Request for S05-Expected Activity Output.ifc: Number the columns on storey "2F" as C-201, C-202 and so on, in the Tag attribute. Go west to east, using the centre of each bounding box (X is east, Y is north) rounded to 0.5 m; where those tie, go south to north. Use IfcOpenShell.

First a look at what the model holds.

```python
import ifcopenshell
import ifcopenshell.util.element
import ifcopenshell.util.placement

model = ifcopenshell.open("S05-Expected Activity Output.ifc")
print(model.schema)
storey = next(s for s in model.by_type("IfcBuildingStorey") if s.Name == "2F")
columns = [e for e in ifcopenshell.util.element.get_decomposition(storey) if e.is_a("IfcColumn")]
for e in sorted(columns, key=lambda e: e.id()):
    origin = ifcopenshell.util.placement.get_local_placement(e.ObjectPlacement)[:3, 3]
    print(e.id(), e.Tag, e.Name, origin.round(2) + 0.0, sep=" | ")
```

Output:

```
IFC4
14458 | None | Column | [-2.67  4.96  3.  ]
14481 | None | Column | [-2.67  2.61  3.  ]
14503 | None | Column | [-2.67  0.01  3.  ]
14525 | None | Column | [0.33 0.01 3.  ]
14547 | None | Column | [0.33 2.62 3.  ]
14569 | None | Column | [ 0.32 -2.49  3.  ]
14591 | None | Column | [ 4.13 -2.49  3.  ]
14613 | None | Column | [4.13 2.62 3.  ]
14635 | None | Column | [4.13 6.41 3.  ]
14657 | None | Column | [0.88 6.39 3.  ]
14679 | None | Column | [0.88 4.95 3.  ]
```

```python
import ifcopenshell
import ifcopenshell.geom
import ifcopenshell.util.element
import ifcopenshell.util.shape

model = ifcopenshell.open("S05-Expected Activity Output.ifc")
settings = ifcopenshell.geom.settings()
settings.set("use-world-coords", True)


def centre(element):
    shape = ifcopenshell.geom.create_shape(settings, element)
    return ifcopenshell.util.shape.get_bbox_centroid(shape.geometry)


storey = next(s for s in model.by_type("IfcBuildingStorey") if s.Name == "2F")
columns = [e for e in ifcopenshell.util.element.get_decomposition(storey) if e.is_a("IfcColumn")]

# Insertion points can sit at a corner or the storey origin, so sort by the geometry (in metres).
centres = {e: centre(e) for e in columns}
columns.sort(key=lambda e: (round(centres[e][0] / 0.5), centres[e][1]))

for i, e in enumerate(columns, start=1):
    number = f"C-2{i:02d}"
    e.Tag = number
    print(e.id(), number)

model.write("S05-Expected Activity Output_edited.ifc")
```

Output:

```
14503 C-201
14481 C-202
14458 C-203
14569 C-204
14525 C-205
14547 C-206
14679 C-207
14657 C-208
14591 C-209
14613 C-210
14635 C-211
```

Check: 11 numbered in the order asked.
